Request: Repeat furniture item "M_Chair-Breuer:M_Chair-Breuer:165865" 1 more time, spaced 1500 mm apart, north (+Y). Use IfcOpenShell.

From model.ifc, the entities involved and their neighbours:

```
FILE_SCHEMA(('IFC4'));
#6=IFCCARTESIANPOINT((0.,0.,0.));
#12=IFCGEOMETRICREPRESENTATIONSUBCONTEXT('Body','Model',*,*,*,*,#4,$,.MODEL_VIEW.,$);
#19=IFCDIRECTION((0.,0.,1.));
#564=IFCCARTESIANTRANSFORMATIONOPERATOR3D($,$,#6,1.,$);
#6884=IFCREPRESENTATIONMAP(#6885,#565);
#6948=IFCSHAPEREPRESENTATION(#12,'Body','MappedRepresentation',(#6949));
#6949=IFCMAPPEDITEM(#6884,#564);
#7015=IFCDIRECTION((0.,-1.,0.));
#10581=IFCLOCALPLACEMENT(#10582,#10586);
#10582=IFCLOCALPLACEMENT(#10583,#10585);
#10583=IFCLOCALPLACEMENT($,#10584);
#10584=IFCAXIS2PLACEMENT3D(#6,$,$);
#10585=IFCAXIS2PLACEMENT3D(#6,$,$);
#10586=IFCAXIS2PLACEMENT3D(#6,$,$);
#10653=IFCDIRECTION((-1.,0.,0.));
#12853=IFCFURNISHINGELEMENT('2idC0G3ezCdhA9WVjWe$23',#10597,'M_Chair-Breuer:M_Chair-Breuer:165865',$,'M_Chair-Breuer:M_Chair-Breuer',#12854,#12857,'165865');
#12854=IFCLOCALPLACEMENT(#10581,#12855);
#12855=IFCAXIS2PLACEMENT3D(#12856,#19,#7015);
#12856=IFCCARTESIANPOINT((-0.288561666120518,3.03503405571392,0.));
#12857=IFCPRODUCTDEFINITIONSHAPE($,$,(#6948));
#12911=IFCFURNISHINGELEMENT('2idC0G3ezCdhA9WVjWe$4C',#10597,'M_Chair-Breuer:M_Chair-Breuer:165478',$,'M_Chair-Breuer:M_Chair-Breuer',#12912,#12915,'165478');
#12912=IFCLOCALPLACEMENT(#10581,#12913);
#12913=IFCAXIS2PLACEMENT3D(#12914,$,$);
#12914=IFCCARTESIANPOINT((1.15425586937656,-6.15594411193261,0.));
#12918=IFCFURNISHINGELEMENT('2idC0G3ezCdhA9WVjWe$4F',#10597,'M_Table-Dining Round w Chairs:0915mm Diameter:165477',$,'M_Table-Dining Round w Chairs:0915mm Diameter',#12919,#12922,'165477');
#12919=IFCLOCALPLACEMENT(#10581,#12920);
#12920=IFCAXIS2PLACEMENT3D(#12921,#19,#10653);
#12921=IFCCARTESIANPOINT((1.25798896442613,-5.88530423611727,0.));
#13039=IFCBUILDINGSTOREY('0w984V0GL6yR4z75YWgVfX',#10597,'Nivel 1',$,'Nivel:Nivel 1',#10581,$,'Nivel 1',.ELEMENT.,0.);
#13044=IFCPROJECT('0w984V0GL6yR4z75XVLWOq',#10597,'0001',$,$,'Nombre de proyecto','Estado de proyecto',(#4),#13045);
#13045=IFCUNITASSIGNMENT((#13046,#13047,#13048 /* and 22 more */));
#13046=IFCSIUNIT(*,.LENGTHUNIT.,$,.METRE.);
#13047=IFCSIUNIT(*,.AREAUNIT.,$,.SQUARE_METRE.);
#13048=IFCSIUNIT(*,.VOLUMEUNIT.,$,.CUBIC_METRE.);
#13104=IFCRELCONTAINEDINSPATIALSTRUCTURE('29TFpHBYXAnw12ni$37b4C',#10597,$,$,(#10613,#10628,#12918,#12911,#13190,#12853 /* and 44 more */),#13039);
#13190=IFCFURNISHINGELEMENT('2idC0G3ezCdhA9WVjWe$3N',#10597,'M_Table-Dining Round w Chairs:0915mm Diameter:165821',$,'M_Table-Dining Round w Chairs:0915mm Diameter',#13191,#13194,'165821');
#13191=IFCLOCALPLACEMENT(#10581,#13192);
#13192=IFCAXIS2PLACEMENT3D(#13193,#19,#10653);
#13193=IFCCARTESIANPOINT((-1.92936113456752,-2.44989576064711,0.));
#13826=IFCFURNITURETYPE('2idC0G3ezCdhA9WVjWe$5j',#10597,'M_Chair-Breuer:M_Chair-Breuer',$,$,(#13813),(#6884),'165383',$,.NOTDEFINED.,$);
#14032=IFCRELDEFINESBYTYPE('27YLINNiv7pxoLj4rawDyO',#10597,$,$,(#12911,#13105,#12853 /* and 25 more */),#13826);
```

```python
import numpy as np
import ifcopenshell
import ifcopenshell.api.geometry
import ifcopenshell.api.root
import ifcopenshell.util.element
import ifcopenshell.util.placement

model = ifcopenshell.open("model.ifc")


def reuse_history(source, copy):
    """copy_class also copies each property set's owner history, people and application; keep the originals."""
    for rel in copy.IsDefinedBy:
        if rel.is_a("IfcRelDefinesByProperties") and (history := rel.RelatingPropertyDefinition.OwnerHistory):
            rel.RelatingPropertyDefinition.OwnerHistory = source.OwnerHistory
            ifcopenshell.util.element.remove_deep2(model, history)


source = model.by_guid("2idC0G3ezCdhA9WVjWe$23")
base = ifcopenshell.util.placement.get_local_placement(source.ObjectPlacement)
step = np.array([0.0, 1.0, 0.0]) * 1.5

for i in range(1, 2):
    copy = ifcopenshell.api.root.copy_class(model, product=source)
    copy.Representation = ifcopenshell.util.element.copy_deep(
        model, source.Representation, exclude=["IfcGeometricRepresentationContext", "IfcRepresentationMap"]
    )
    copy.Name = "M_Chair-Breuer:M_Chair-Breuer"
    copy.Tag = None
    reuse_history(source, copy)
    matrix = base.copy()
    matrix[:3, 3] += i * step
    print("added at", matrix[:3, 3].round(3) + 0.0)
    ifcopenshell.api.geometry.edit_object_placement(model, product=copy, matrix=matrix, is_si=False)

model.write("model_edited.ifc")
```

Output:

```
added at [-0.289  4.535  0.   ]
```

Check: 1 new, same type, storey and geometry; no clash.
